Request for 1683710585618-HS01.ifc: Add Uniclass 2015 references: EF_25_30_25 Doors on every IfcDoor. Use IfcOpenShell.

First a look at what the model holds.

```python
import ifcopenshell

model = ifcopenshell.open("1683710585618-HS01.ifc")
print(model.schema)
print("classifications:", [c.Name for c in model.by_type("IfcClassification")])
for ifc_class in ("IfcDoor", "IfcRoof", "IfcStair", "IfcWall", "IfcWindow"):
    print(ifc_class, len(model.by_type(ifc_class)))
```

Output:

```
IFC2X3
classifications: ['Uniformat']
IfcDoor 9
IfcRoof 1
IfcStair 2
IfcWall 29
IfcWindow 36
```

```python
import ifcopenshell
import ifcopenshell.api.classification

model = ifcopenshell.open("1683710585618-HS01.ifc")

# IFC2X3 requires Source and Edition and has no link from the project to the system.
system = model.create_entity("IfcClassification", Source="NBS", Edition="2015", Name="Uniclass 2015")

codes = {
    "IfcDoor": ("EF_25_30_25", "Doors"),
}
for ifc_class, (code, name) in codes.items():
    products = model.by_type(ifc_class)
    ifcopenshell.api.classification.add_reference(
        model, products=products, classification=system, identification=code, name=name
    )
    print(code, len(products))

model.write("1683710585618-HS01_edited.ifc")
```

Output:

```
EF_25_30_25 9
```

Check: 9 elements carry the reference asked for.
